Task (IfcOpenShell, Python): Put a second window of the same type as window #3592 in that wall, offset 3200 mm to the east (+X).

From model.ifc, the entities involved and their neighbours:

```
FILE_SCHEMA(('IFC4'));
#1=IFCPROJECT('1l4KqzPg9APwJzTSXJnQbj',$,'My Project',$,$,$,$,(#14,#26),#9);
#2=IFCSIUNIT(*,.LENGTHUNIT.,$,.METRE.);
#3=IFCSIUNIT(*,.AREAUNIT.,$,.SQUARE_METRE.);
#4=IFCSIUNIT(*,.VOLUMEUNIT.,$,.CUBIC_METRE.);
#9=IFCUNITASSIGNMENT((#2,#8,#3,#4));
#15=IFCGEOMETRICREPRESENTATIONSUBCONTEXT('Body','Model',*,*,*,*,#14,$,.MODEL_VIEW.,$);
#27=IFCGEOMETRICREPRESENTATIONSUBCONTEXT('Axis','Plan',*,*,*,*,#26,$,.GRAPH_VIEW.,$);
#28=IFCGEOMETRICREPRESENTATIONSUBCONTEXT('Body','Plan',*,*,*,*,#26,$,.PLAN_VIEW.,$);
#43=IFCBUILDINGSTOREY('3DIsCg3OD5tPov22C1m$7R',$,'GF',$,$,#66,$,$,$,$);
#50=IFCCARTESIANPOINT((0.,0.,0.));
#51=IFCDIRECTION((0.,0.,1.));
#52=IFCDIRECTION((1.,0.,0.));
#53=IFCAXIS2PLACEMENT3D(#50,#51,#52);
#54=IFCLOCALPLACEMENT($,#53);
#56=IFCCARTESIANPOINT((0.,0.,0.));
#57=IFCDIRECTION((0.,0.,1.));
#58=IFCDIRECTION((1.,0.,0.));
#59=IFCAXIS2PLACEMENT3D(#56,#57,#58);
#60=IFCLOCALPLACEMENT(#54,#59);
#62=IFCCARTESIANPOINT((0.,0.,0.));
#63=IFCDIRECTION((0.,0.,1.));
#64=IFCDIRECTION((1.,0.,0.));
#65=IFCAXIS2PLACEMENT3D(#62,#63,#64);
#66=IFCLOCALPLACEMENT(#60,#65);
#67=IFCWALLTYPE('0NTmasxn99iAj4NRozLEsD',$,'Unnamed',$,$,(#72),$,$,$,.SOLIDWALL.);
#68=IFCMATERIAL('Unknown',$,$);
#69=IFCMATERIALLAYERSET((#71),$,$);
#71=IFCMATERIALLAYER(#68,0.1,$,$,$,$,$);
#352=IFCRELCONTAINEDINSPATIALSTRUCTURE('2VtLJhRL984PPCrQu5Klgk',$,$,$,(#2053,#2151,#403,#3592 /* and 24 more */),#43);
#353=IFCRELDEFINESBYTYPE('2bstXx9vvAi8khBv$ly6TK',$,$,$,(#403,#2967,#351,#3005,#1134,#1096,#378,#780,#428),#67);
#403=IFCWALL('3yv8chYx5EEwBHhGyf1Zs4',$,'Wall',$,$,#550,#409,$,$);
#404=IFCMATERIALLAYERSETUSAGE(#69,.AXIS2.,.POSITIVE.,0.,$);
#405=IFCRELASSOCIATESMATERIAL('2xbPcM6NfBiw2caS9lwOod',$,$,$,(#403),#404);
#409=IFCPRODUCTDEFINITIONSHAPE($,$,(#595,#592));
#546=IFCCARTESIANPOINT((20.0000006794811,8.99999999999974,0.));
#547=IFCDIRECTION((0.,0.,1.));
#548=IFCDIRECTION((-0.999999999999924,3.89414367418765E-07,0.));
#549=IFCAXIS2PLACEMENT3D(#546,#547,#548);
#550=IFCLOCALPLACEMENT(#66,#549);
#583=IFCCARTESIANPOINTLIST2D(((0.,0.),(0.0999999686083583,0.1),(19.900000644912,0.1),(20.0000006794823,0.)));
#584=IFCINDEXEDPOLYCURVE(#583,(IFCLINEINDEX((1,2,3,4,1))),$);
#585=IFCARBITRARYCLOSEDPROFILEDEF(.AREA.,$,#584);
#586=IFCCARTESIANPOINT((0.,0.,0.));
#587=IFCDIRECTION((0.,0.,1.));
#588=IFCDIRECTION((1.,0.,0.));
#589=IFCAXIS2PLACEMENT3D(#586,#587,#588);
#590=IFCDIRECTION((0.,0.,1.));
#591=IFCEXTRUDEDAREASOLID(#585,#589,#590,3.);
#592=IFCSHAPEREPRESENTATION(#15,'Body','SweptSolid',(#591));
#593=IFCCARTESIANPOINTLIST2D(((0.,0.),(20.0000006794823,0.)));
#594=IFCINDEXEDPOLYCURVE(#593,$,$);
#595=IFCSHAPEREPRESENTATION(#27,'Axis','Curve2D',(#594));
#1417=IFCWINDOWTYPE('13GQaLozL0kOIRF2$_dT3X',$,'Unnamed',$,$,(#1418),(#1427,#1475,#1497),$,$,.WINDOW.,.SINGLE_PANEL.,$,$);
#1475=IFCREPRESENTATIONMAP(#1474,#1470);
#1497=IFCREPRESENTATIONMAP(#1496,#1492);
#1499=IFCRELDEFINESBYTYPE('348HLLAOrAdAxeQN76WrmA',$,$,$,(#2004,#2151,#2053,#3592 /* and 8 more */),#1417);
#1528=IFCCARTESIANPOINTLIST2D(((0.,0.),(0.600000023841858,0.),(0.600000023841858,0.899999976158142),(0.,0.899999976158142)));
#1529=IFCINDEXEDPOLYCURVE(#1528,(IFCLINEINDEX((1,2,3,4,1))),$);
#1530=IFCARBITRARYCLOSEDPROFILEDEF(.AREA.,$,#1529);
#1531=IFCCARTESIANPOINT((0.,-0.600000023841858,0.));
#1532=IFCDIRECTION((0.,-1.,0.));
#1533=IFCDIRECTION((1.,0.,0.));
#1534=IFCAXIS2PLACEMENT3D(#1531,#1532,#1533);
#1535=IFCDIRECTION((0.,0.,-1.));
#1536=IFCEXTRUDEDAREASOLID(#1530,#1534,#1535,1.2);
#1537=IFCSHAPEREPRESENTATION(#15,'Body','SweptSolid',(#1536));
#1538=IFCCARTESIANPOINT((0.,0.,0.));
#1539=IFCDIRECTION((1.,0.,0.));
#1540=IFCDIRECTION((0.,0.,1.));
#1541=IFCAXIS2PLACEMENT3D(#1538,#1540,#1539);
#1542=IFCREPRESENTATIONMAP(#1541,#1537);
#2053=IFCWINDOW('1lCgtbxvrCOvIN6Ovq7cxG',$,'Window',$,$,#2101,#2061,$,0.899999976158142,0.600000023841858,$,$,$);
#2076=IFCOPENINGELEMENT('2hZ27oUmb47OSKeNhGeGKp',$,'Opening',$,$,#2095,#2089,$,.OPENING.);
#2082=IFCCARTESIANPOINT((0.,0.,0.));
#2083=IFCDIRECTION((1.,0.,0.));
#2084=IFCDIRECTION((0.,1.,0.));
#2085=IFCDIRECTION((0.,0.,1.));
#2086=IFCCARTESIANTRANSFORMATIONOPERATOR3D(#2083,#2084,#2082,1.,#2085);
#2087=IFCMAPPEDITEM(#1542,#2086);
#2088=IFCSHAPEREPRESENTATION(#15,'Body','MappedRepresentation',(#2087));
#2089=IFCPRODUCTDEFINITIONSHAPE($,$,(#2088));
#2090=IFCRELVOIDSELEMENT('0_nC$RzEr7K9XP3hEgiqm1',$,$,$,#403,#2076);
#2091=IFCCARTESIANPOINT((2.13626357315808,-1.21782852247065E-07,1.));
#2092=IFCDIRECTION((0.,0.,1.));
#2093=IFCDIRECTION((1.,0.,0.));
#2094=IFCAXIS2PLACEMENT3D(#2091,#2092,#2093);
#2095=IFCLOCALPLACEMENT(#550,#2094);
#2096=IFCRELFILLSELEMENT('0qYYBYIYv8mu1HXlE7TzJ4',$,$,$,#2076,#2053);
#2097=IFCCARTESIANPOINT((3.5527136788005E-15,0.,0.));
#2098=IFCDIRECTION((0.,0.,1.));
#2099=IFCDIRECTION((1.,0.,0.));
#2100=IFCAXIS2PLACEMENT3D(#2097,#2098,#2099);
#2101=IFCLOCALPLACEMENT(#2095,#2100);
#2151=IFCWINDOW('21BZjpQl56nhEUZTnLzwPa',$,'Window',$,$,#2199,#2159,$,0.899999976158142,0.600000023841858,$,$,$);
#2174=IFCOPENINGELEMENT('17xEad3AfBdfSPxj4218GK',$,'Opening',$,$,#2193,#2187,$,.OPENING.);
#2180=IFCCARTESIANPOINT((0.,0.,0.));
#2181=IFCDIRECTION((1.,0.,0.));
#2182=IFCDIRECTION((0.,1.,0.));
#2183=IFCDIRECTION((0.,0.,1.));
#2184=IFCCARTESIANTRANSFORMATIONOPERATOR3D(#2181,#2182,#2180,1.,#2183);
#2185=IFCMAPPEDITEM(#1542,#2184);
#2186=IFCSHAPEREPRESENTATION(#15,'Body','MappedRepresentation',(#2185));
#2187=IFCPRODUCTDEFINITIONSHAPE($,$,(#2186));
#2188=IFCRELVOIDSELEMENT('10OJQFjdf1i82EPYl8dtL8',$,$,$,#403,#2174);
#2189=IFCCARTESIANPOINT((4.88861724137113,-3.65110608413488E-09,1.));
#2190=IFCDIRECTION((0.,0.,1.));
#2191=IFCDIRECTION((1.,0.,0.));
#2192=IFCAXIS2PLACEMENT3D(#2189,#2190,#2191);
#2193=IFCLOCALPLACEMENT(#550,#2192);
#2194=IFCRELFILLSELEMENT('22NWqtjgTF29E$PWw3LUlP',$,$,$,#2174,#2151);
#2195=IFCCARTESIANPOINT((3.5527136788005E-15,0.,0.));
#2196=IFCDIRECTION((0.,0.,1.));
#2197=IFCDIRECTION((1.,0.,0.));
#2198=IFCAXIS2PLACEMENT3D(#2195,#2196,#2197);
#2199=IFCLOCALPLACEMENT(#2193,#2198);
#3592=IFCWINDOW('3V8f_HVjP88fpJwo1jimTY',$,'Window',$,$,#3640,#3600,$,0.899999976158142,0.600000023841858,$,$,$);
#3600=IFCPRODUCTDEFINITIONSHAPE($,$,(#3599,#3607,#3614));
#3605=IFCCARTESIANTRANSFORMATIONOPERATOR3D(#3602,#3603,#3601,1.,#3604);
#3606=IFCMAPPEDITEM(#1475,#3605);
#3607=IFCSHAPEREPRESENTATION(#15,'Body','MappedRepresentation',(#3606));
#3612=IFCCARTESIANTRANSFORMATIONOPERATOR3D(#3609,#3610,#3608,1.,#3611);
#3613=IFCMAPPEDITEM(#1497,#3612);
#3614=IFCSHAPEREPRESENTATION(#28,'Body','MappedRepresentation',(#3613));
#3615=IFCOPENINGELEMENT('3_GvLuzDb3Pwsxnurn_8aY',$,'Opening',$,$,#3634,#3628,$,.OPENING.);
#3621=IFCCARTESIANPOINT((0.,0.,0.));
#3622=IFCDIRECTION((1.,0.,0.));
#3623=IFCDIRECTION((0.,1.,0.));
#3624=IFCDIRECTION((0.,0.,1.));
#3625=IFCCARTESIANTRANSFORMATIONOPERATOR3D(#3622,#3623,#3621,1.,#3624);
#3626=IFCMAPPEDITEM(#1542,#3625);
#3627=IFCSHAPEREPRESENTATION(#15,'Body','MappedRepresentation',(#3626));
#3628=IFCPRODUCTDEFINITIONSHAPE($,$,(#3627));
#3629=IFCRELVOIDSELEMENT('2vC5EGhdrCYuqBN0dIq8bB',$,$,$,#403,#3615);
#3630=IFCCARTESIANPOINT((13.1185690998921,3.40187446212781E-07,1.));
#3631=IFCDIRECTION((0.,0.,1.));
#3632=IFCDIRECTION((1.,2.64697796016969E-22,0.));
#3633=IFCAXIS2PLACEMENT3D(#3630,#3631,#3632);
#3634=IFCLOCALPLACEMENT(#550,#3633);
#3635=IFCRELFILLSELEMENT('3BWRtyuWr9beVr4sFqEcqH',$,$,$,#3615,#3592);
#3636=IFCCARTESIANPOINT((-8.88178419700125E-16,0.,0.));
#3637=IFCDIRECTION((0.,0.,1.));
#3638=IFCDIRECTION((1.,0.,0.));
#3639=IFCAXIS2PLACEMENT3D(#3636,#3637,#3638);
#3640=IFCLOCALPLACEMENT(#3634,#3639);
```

```python
import ifcopenshell
import ifcopenshell.api.feature
import ifcopenshell.api.geometry
import ifcopenshell.api.root
import ifcopenshell.geom
import ifcopenshell.util.element
import ifcopenshell.util.placement
import ifcopenshell.util.shape
import ifcopenshell.util.unit

model = ifcopenshell.open("model.ifc")
unit_scale = ifcopenshell.util.unit.calculate_unit_scale(model)
settings = ifcopenshell.geom.settings()


def volume(element):
    """Net volume in cubic metres, openings subtracted."""
    shape = ifcopenshell.geom.create_shape(settings, element)
    return ifcopenshell.util.shape.get_volume(shape.geometry)


window = model.by_guid("3V8f_HVjP88fpJwo1jimTY")
opening = window.FillsVoids[0].RelatingOpeningElement
wall = opening.VoidsElements[0].RelatingBuildingElement
before = volume(wall)
shift = ifcopenshell.util.placement.get_local_placement(wall.ObjectPlacement)[:3, 0] * -3.2 / unit_scale

# copy_class copies the void relationship, type, container and properties, but no geometry.
new_opening = ifcopenshell.api.root.copy_class(model, product=opening)
new_opening.Representation = ifcopenshell.util.element.copy_deep(
    model, opening.Representation, exclude=["IfcGeometricRepresentationContext", "IfcRepresentationMap"]
)
new_window = ifcopenshell.api.root.copy_class(model, product=window)
new_window.Representation = ifcopenshell.util.element.copy_deep(
    model, window.Representation, exclude=["IfcGeometricRepresentationContext", "IfcRepresentationMap"]
)
ifcopenshell.api.feature.add_filling(model, opening=new_opening, element=new_window)

for old, new in ((opening, new_opening), (window, new_window)):
    matrix = ifcopenshell.util.placement.get_local_placement(old.ObjectPlacement)
    matrix[:3, 3] += shift
    ifcopenshell.api.geometry.edit_object_placement(model, product=new, matrix=matrix, is_si=False)

after = volume(wall)

print(f"wall volume {before:.3f} -> {after:.3f} m3")

model.write("model_updated.ifc")
```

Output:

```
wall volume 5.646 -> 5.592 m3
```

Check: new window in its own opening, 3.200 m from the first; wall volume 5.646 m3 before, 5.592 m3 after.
